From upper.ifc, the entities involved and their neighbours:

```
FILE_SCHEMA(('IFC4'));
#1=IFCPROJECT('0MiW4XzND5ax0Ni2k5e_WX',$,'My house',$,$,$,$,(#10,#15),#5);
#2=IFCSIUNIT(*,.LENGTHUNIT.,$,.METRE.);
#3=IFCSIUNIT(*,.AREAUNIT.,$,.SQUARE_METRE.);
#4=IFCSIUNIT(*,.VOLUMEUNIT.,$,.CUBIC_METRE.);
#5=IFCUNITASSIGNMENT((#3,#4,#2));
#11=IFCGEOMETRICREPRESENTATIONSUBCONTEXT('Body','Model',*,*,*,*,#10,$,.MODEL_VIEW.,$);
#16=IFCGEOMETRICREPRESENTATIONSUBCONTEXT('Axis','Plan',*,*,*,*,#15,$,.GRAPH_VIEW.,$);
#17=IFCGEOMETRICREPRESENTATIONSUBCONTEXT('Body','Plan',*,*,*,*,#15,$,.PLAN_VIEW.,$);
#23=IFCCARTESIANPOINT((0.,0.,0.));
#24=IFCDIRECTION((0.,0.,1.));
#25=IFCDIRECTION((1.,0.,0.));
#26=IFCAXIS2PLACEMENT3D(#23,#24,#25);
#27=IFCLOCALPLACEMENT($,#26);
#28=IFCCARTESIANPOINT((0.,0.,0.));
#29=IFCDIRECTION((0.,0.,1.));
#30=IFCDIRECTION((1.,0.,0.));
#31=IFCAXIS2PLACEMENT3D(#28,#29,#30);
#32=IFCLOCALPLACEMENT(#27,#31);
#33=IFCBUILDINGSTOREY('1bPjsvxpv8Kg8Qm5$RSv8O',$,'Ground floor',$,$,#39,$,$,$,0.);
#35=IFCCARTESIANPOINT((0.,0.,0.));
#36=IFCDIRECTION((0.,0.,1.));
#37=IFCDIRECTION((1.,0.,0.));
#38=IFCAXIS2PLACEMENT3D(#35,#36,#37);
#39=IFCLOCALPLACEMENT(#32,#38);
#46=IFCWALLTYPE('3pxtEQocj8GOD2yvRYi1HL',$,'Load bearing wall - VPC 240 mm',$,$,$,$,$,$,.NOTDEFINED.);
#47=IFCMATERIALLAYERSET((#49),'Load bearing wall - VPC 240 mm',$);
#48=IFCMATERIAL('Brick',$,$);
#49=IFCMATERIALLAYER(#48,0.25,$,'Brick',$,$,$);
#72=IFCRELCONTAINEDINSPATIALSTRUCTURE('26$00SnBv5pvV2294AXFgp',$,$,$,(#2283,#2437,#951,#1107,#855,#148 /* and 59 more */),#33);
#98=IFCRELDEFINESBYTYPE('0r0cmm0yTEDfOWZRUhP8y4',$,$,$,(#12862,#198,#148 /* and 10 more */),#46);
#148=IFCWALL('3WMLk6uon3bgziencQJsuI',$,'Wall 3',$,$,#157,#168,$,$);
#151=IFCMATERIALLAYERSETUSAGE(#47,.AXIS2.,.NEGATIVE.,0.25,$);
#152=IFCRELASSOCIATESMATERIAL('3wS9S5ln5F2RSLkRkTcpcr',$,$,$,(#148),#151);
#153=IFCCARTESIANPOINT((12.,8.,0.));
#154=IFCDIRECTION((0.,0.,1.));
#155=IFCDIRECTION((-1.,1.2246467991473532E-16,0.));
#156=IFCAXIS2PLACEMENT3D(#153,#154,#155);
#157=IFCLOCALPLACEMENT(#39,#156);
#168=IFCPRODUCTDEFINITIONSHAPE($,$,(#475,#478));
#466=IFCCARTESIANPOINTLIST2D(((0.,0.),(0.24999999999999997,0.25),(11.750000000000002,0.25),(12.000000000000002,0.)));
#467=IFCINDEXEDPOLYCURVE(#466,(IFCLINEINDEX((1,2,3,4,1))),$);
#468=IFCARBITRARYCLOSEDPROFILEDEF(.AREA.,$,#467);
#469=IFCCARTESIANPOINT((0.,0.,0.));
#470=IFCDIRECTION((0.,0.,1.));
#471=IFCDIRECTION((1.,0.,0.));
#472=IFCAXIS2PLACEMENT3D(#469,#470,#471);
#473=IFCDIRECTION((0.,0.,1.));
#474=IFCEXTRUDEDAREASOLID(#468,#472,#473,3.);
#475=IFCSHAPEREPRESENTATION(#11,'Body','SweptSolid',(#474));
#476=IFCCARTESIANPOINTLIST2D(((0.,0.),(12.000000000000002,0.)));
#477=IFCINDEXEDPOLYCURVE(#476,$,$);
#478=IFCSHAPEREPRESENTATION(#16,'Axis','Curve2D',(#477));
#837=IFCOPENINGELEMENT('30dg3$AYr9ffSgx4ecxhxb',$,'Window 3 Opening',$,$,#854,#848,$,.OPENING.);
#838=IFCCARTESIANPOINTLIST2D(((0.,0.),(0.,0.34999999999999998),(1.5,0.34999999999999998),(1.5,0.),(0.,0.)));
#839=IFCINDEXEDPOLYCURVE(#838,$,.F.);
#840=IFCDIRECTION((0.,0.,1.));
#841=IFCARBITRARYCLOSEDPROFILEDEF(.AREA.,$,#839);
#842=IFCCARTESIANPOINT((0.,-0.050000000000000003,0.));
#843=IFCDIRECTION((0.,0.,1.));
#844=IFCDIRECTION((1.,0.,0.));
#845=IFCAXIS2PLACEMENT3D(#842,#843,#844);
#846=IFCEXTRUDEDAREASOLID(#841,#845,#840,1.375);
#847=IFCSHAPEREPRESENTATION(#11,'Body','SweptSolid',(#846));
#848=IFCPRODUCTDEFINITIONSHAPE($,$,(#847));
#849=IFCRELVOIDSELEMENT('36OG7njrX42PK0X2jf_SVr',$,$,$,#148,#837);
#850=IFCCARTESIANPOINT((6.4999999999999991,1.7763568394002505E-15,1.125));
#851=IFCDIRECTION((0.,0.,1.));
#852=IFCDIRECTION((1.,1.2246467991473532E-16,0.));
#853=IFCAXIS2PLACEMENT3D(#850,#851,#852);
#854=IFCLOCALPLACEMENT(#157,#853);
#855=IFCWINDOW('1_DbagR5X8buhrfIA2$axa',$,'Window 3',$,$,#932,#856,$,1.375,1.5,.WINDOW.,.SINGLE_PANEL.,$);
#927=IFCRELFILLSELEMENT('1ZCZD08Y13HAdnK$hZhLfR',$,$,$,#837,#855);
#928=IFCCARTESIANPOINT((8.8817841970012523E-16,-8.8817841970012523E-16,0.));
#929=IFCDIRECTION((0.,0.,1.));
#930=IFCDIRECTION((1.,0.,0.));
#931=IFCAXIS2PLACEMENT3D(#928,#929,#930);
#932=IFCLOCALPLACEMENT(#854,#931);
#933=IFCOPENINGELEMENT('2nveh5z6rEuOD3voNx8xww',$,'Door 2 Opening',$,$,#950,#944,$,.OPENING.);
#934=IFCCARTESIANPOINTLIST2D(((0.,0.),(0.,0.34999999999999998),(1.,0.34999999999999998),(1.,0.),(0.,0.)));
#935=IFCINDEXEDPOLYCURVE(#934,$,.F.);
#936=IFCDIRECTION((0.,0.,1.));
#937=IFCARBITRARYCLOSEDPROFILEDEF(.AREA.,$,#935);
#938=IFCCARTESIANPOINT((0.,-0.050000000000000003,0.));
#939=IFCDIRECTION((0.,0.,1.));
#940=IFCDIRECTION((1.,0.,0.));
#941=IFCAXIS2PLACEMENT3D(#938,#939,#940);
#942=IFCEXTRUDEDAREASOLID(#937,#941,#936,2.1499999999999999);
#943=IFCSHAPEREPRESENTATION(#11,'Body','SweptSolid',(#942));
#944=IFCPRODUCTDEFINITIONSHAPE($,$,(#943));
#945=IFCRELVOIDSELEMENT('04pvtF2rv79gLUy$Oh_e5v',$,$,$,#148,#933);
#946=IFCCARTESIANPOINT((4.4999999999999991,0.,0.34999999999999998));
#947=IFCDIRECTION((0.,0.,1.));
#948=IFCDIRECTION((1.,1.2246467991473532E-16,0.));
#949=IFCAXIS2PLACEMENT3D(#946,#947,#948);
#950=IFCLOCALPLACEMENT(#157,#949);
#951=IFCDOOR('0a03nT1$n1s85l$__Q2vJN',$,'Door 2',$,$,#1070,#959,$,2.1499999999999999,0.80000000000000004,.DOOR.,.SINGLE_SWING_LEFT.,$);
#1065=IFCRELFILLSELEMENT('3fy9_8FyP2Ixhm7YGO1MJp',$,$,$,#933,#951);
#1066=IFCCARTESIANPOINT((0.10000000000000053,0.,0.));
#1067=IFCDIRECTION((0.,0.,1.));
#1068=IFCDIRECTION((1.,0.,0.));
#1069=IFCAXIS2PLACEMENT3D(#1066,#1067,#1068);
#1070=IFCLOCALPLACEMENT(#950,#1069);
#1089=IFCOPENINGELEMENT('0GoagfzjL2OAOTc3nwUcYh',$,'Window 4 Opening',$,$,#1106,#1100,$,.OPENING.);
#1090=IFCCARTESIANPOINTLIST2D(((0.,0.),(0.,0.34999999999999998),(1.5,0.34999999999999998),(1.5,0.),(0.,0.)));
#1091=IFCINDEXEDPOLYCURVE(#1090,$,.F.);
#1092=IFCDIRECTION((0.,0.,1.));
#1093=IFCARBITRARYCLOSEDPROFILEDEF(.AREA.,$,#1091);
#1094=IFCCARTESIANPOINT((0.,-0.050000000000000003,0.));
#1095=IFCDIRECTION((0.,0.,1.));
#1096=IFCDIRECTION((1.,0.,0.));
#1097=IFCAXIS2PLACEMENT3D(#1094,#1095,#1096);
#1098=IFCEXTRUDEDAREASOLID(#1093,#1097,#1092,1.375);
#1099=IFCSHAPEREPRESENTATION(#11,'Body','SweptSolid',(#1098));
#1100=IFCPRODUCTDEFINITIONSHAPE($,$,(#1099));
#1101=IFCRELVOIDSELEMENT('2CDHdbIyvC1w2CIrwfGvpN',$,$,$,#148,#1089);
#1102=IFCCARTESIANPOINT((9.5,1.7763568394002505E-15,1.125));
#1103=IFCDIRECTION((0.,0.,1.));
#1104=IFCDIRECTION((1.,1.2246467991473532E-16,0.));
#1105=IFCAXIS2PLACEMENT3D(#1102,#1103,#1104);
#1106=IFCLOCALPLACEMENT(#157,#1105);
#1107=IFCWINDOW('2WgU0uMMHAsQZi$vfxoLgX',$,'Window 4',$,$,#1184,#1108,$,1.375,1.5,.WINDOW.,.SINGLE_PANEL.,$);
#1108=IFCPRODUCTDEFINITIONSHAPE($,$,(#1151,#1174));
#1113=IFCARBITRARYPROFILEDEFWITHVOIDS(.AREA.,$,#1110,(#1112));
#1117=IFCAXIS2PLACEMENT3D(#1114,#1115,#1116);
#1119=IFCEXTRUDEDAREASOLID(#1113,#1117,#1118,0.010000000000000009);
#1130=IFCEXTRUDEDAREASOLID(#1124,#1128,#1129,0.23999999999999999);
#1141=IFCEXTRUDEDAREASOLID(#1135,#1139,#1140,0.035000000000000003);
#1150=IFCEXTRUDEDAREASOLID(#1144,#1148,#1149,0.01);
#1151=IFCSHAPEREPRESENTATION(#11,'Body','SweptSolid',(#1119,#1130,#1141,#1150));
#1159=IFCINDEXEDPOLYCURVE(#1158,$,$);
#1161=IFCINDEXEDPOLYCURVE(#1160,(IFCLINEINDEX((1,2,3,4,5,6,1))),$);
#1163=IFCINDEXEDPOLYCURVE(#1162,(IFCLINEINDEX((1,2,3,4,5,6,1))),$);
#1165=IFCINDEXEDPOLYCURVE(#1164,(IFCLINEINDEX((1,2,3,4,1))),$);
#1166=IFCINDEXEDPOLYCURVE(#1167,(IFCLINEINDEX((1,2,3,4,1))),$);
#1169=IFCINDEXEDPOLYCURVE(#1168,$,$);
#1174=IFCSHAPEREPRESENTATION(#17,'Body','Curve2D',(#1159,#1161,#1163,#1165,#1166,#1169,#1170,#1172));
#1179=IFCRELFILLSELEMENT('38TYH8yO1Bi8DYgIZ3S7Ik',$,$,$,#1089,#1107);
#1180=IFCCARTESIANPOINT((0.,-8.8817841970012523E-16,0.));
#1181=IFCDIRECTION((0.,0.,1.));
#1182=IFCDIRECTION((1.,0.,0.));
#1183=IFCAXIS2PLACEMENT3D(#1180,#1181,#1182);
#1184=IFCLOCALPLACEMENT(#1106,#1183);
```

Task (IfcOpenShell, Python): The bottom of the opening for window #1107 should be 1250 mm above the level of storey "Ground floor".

```python
import numpy as np
import ifcopenshell
import ifcopenshell.api.geometry
import ifcopenshell.geom
import ifcopenshell.util.element
import ifcopenshell.util.placement
import ifcopenshell.util.shape
import ifcopenshell.util.unit

model = ifcopenshell.open("upper.ifc")
unit_scale = ifcopenshell.util.unit.calculate_unit_scale(model)

window = model.by_guid("2WgU0uMMHAsQZi$vfxoLgX")
opening = window.FillsVoids[0].RelatingOpeningElement
storey = ifcopenshell.util.element.get_container(window, ifc_class="IfcBuildingStorey")
level = ifcopenshell.util.placement.get_local_placement(storey.ObjectPlacement)[2, 3]

# The opening's origin need not be at the sill, so measure its lowest point.
shape = ifcopenshell.geom.create_shape(ifcopenshell.geom.settings(), opening)
bottom = ifcopenshell.util.shape.get_shape_bottom_elevation(shape, shape.geometry) / unit_scale
dz = level + 1.25 - bottom

shift = np.array([0.0, 0.0, dz])
# The window is placed relative to its opening, so it follows when the opening moves.
matrix = ifcopenshell.util.placement.get_local_placement(opening.ObjectPlacement)
matrix[:3, 3] += shift
ifcopenshell.api.geometry.edit_object_placement(
    model, product=opening, matrix=matrix, is_si=False, should_transform_children=True
)

print(f"moved by {dz * unit_scale:+.3f} m")

model.write("upper_edited.ifc")
```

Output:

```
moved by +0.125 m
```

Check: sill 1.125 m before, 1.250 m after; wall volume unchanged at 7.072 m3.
